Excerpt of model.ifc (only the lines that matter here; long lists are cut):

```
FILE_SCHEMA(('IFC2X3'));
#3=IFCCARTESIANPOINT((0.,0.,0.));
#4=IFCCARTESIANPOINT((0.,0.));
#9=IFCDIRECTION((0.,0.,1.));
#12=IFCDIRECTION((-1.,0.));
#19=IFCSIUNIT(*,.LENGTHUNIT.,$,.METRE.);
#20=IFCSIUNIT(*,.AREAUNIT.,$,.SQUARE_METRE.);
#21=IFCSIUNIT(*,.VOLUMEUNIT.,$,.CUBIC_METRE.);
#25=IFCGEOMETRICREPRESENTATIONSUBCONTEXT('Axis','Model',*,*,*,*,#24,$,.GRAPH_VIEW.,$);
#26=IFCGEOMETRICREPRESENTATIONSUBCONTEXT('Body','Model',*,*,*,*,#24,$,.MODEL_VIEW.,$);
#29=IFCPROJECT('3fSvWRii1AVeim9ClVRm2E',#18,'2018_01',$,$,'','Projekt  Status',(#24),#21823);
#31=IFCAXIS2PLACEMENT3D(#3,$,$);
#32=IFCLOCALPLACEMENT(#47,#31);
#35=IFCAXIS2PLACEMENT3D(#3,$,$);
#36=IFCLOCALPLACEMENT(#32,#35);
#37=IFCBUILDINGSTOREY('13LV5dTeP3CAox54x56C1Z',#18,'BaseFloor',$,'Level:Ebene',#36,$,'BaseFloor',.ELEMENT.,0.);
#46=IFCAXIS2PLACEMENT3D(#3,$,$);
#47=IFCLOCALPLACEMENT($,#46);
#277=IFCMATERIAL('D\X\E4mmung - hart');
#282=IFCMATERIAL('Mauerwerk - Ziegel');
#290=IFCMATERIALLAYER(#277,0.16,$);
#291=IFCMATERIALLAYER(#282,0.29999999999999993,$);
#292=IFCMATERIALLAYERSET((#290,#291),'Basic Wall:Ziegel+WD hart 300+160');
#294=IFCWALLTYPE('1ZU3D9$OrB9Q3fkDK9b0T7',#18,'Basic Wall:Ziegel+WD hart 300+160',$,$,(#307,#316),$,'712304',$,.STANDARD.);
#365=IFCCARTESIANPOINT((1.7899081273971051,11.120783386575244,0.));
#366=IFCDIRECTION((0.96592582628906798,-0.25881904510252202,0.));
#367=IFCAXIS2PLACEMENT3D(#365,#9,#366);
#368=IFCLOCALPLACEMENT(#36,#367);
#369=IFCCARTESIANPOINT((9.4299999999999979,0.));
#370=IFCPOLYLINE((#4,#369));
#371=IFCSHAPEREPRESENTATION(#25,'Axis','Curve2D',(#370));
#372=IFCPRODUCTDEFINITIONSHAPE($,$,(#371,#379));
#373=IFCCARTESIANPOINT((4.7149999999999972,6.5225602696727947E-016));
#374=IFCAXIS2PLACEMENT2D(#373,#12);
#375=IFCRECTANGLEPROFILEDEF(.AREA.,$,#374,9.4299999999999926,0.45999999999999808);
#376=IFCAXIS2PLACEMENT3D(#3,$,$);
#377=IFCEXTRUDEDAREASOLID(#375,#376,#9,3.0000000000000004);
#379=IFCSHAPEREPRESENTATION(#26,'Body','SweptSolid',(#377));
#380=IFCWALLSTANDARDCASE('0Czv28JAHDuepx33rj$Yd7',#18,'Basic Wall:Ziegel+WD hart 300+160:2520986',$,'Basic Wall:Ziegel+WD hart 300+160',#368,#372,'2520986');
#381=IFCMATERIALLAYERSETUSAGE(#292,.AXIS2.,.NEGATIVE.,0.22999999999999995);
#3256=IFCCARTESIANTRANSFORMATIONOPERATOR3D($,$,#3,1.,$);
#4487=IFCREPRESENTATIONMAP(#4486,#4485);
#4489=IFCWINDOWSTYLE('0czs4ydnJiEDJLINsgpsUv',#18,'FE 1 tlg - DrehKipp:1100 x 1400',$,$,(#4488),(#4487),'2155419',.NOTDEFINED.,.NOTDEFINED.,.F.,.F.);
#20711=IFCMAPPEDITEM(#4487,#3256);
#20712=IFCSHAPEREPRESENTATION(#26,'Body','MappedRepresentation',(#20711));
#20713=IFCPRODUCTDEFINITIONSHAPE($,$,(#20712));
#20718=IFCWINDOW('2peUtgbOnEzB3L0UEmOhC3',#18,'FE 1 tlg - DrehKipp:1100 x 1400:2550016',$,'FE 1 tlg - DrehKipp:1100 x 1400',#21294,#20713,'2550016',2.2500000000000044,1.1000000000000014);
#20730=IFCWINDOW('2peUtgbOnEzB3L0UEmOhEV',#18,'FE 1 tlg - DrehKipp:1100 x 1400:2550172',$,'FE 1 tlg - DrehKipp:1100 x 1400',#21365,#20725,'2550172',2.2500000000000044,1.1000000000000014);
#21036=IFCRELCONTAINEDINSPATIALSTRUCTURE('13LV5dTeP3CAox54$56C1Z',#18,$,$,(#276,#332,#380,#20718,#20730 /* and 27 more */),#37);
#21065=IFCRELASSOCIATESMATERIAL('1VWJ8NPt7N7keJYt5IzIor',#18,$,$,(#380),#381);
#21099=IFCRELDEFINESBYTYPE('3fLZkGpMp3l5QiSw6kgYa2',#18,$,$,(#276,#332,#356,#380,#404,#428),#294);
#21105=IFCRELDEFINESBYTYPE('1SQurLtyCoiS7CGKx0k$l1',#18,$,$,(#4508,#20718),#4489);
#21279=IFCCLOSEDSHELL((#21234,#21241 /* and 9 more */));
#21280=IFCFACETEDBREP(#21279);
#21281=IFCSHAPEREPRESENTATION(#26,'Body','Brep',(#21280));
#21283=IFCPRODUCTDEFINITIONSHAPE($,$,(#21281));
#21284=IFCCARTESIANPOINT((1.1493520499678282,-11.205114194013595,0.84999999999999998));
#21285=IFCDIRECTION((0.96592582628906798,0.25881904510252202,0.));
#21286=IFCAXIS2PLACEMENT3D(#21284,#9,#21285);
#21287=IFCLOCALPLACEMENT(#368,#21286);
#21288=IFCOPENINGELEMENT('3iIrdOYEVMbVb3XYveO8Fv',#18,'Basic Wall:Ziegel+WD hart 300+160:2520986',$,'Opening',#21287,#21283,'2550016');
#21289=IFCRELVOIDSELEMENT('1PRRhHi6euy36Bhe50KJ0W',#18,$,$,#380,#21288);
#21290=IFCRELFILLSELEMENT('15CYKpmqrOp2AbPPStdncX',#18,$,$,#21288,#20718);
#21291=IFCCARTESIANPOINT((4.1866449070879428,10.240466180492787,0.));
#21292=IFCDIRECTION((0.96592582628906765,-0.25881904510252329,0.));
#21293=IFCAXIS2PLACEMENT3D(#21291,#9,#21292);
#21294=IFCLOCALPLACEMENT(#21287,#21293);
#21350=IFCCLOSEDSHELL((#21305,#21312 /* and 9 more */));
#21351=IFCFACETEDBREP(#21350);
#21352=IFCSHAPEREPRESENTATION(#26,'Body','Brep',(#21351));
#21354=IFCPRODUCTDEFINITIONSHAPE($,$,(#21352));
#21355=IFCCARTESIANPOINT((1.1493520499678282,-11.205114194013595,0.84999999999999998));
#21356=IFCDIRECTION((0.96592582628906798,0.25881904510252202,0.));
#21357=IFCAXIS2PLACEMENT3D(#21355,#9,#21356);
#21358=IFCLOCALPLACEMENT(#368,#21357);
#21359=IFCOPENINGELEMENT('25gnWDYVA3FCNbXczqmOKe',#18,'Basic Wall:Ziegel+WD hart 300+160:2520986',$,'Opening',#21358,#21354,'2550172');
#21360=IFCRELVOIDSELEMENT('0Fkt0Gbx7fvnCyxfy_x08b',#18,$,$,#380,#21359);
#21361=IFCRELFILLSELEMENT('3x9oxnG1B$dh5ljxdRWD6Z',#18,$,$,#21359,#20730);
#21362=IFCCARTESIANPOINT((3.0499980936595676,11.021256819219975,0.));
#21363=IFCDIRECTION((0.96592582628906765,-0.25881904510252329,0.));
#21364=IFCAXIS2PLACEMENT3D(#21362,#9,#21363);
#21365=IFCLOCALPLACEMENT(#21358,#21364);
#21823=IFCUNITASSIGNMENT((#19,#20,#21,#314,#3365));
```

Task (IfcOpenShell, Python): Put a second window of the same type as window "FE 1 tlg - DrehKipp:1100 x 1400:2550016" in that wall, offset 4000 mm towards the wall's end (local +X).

```python
import ifcopenshell
import ifcopenshell.api.feature
import ifcopenshell.api.geometry
import ifcopenshell.api.root
import ifcopenshell.geom
import ifcopenshell.util.element
import ifcopenshell.util.placement
import ifcopenshell.util.shape
import ifcopenshell.util.unit

model = ifcopenshell.open("model.ifc")
unit_scale = ifcopenshell.util.unit.calculate_unit_scale(model)
settings = ifcopenshell.geom.settings()


def volume(element):
    """Net volume in cubic metres, openings subtracted."""
    shape = ifcopenshell.geom.create_shape(settings, element)
    return ifcopenshell.util.shape.get_volume(shape.geometry)


def reuse_history(source, copy):
    """copy_class also copies each property set's owner history, people and application; keep the originals."""
    for rel in copy.IsDefinedBy:
        if rel.is_a("IfcRelDefinesByProperties") and (history := rel.RelatingPropertyDefinition.OwnerHistory):
            rel.RelatingPropertyDefinition.OwnerHistory = source.OwnerHistory
            ifcopenshell.util.element.remove_deep2(model, history)


window = model.by_guid("2peUtgbOnEzB3L0UEmOhC3")
opening = window.FillsVoids[0].RelatingOpeningElement
wall = opening.VoidsElements[0].RelatingBuildingElement
before = volume(wall)
shift = ifcopenshell.util.placement.get_local_placement(wall.ObjectPlacement)[:3, 0] * 4 / unit_scale

# copy_class copies the void relationship, type, container and properties, but no geometry.
new_opening = ifcopenshell.api.root.copy_class(model, product=opening)
new_opening.Representation = ifcopenshell.util.element.copy_deep(
    model, opening.Representation, exclude=["IfcGeometricRepresentationContext", "IfcRepresentationMap"]
)
new_opening.Name = "Basic Wall:Ziegel+WD hart 300+160"
new_opening.Tag = None
new_window = ifcopenshell.api.root.copy_class(model, product=window)
new_window.Representation = ifcopenshell.util.element.copy_deep(
    model, window.Representation, exclude=["IfcGeometricRepresentationContext", "IfcRepresentationMap"]
)
new_window.Name = "FE 1 tlg - DrehKipp:1100 x 1400"
new_window.Tag = None
reuse_history(window, new_window)
fills = ifcopenshell.api.feature.add_filling(model, opening=new_opening, element=new_window)
fills.OwnerHistory = new_window.OwnerHistory  # required in IFC2X3

for old, new in ((opening, new_opening), (window, new_window)):
    matrix = ifcopenshell.util.placement.get_local_placement(old.ObjectPlacement)
    matrix[:3, 3] += shift
    ifcopenshell.api.geometry.edit_object_placement(model, product=new, matrix=matrix, is_si=False)

after = volume(wall)

print(f"wall volume {before:.3f} -> {after:.3f} m3")

model.write("model_v2.ifc")
```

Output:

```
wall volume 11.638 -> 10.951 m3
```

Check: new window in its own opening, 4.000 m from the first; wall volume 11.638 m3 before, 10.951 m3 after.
